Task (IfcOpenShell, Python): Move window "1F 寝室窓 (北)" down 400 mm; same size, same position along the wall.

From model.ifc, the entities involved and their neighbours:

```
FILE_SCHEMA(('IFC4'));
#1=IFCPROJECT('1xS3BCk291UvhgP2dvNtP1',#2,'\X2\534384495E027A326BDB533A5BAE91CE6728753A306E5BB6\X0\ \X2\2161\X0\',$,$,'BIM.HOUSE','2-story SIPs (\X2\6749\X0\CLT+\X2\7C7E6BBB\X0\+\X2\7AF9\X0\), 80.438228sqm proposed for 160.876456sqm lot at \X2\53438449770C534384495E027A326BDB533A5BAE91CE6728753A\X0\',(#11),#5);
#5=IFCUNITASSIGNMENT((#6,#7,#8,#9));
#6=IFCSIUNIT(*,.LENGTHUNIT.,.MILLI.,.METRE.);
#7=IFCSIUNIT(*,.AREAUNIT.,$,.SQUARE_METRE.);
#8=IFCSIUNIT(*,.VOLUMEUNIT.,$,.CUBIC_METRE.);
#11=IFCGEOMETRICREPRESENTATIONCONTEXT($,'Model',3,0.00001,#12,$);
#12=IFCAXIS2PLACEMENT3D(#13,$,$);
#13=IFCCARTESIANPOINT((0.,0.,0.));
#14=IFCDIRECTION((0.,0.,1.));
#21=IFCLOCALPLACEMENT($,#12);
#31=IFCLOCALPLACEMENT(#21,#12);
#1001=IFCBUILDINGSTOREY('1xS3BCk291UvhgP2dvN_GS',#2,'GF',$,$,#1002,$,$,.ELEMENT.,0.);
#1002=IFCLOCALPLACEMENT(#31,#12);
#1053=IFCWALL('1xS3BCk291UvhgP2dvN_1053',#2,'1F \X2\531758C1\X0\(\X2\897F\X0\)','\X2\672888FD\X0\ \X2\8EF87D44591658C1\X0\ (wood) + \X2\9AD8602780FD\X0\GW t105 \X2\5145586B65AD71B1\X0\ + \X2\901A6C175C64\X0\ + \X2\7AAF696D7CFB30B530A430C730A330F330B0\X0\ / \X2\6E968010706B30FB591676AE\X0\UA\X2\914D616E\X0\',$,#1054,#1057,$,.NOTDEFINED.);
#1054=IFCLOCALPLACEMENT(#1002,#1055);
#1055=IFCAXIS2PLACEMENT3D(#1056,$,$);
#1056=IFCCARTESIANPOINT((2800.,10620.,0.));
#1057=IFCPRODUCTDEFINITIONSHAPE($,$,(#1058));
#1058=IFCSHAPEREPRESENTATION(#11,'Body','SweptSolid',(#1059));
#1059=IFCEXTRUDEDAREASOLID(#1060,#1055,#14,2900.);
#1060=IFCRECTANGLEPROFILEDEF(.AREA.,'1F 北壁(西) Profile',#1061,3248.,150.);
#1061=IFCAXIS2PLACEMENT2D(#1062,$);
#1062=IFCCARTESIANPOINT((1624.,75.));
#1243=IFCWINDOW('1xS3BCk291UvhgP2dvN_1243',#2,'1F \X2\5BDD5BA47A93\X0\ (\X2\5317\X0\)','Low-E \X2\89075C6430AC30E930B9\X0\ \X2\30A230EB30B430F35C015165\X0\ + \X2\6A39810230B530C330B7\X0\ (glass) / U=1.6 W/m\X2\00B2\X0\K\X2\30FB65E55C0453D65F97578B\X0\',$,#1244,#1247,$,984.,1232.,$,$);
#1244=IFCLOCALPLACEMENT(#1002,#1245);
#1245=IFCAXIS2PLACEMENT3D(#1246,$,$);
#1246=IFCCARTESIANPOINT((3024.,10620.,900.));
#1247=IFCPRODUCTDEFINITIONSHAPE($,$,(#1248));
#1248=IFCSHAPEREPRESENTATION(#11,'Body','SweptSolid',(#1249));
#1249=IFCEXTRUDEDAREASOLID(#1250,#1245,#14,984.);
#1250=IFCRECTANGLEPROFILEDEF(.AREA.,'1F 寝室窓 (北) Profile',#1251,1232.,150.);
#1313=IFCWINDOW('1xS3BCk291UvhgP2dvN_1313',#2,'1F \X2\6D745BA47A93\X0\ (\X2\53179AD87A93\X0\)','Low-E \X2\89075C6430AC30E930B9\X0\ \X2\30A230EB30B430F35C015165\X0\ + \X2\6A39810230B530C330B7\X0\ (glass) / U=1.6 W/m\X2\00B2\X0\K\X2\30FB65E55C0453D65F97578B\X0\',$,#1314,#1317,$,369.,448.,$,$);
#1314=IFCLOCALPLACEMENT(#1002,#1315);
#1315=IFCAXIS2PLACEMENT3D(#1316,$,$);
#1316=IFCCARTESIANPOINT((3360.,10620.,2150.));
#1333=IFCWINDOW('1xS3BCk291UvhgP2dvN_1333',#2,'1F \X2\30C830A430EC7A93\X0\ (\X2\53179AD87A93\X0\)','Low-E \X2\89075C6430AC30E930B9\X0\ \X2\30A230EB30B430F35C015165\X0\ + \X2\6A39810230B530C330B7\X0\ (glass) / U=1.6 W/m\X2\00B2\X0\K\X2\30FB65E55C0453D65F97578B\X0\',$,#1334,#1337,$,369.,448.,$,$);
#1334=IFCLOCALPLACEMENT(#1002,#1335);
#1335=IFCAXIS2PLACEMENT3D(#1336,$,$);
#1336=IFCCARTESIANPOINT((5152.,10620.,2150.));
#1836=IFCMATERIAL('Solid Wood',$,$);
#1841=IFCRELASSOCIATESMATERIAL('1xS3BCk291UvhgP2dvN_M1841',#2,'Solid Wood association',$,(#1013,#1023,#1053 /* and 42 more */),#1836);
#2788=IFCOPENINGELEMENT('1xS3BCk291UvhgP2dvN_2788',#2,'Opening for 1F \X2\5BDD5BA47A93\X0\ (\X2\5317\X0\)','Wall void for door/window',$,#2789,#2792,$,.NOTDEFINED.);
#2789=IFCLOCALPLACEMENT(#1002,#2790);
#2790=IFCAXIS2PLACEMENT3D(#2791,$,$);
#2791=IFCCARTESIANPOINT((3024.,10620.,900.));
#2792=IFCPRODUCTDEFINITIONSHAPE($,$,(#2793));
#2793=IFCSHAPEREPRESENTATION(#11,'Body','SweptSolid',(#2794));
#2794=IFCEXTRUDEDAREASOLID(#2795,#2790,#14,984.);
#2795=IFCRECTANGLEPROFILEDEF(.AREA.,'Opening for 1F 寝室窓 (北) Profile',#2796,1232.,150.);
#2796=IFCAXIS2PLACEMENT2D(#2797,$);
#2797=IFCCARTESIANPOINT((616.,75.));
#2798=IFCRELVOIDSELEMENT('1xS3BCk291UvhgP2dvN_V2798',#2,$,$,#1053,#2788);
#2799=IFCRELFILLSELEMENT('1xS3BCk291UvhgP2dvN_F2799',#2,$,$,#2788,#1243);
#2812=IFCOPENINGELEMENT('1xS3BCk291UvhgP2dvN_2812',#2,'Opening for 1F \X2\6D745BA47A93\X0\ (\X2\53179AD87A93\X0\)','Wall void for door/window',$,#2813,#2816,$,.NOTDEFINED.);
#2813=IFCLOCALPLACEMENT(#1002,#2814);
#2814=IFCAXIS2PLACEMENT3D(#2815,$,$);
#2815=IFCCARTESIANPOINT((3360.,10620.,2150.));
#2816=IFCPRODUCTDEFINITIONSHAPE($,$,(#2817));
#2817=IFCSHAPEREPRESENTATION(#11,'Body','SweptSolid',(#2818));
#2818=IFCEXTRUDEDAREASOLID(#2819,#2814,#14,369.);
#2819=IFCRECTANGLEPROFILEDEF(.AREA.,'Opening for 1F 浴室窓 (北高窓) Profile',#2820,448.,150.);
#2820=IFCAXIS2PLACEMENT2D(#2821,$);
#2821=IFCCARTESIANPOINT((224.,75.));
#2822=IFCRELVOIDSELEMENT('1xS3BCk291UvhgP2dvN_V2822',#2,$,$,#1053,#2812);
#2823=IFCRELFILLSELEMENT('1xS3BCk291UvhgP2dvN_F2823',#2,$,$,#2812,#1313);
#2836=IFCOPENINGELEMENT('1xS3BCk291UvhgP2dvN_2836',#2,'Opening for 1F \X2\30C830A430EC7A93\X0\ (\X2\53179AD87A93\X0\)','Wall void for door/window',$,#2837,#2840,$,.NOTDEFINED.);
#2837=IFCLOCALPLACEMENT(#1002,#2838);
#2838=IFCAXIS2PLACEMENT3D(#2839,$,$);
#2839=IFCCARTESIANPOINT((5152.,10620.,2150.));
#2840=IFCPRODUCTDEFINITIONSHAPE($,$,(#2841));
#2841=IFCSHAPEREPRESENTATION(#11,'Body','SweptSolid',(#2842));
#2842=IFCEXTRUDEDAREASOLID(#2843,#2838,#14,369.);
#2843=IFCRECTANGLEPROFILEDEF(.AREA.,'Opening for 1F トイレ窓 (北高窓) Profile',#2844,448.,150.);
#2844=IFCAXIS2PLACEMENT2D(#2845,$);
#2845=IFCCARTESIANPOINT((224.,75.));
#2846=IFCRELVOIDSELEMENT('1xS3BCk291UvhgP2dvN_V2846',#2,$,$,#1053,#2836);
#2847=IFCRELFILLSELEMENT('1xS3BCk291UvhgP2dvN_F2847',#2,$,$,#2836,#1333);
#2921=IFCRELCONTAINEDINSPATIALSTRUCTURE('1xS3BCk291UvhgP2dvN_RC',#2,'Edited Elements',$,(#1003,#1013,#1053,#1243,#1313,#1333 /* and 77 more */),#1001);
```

```python
import numpy as np
import ifcopenshell
import ifcopenshell.api.geometry
import ifcopenshell.util.placement
import ifcopenshell.util.unit

model = ifcopenshell.open("model.ifc")
unit_scale = ifcopenshell.util.unit.calculate_unit_scale(model)

window = model.by_guid("1xS3BCk291UvhgP2dvN_1243")
opening = window.FillsVoids[0].RelatingOpeningElement
dz = -0.4 / unit_scale

shift = np.array([0.0, 0.0, dz])
# The window is not placed relative to its opening, so move both.
for product in (opening, window):
    matrix = ifcopenshell.util.placement.get_local_placement(product.ObjectPlacement)
    matrix[:3, 3] += shift
    ifcopenshell.api.geometry.edit_object_placement(model, product=product, matrix=matrix, is_si=False)

print(f"moved by {dz * unit_scale:+.3f} m")

model.write("model_edited.ifc")
```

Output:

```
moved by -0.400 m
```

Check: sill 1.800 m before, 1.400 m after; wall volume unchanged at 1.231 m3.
